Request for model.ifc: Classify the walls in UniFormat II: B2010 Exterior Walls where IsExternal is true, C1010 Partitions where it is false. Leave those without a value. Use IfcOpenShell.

First a look at what the model holds.

```python
import ifcopenshell
import ifcopenshell.util.element

model = ifcopenshell.open("model.ifc")
print(model.schema)
print("classifications:", [c.Name for c in model.by_type("IfcClassification")])
values = [ifcopenshell.util.element.get_pset(e, "Pset_WallCommon", "IsExternal") for e in model.by_type("IfcWall")]
for value in (True, False, None):
    print("IsExternal", value, values.count(value))
```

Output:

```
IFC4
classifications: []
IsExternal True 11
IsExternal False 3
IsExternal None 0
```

```python
import ifcopenshell
import ifcopenshell.api.classification
import ifcopenshell.util.element

model = ifcopenshell.open("model.ifc")

system = ifcopenshell.api.classification.add_classification(model, classification="UniFormat II")

walls = model.by_type("IfcWall")
external = {e: ifcopenshell.util.element.get_pset(e, "Pset_WallCommon", "IsExternal") for e in walls}
for flag, code, name in ((True, "B2010", "Exterior Walls"), (False, "C1010", "Partitions")):
    products = [e for e in walls if external[e] is flag]
    ifcopenshell.api.classification.add_reference(
        model, products=products, classification=system, identification=code, name=name
    )
    print(code, len(products))

model.write("model_edited.ifc")
```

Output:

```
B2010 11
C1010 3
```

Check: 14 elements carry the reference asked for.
